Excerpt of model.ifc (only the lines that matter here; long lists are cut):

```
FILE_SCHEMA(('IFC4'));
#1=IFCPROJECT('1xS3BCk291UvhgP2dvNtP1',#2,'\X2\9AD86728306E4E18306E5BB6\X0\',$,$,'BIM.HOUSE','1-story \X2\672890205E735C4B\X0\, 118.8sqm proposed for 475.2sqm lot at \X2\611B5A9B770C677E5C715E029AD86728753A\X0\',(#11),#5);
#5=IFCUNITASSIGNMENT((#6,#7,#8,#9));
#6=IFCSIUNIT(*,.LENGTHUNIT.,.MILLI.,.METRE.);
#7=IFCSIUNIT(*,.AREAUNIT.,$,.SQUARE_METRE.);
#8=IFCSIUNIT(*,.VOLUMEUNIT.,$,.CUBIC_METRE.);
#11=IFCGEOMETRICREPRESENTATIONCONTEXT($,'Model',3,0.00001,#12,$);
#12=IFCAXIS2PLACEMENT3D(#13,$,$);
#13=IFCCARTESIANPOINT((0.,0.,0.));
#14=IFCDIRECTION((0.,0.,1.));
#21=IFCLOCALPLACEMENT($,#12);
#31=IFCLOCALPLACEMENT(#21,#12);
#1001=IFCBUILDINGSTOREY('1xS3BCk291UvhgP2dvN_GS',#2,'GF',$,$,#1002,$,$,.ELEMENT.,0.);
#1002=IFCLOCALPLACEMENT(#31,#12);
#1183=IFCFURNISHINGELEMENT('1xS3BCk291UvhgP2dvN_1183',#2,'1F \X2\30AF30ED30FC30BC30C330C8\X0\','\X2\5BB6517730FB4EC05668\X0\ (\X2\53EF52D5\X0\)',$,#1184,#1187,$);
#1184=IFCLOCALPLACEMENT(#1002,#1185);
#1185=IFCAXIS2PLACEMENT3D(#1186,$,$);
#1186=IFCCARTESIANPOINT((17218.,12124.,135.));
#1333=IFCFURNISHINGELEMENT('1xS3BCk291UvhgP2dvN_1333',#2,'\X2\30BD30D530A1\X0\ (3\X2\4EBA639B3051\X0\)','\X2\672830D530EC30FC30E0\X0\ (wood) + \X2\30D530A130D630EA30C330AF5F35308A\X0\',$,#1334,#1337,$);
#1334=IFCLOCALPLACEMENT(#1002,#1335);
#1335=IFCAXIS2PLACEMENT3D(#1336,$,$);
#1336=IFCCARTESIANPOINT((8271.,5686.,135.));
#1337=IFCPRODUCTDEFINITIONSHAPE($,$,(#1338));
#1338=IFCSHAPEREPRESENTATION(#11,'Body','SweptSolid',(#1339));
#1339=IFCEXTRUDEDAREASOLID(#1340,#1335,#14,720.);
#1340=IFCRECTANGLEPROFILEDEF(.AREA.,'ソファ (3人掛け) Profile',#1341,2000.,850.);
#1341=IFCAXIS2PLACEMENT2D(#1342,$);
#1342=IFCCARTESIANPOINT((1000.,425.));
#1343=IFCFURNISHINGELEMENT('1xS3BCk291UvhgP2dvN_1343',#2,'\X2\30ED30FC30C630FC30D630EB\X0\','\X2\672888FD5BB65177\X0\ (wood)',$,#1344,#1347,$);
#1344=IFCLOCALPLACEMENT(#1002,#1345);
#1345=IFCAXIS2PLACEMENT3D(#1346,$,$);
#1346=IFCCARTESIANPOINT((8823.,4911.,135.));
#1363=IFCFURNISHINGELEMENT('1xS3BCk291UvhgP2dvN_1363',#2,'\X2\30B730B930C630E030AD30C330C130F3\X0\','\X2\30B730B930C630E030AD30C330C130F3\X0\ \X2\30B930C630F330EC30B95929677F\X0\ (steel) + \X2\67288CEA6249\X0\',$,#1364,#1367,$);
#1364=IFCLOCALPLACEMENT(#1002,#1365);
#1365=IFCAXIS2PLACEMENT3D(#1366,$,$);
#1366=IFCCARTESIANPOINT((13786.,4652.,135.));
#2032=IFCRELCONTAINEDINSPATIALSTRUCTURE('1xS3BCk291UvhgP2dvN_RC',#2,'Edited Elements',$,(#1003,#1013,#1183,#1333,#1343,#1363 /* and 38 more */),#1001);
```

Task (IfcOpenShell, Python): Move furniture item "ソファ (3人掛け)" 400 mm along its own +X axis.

```python
import ifcopenshell
import ifcopenshell.api.geometry
import ifcopenshell.util.placement
import ifcopenshell.util.unit

model = ifcopenshell.open("model.ifc")
unit_scale = ifcopenshell.util.unit.calculate_unit_scale(model)

item = model.by_guid("1xS3BCk291UvhgP2dvN_1333")
matrix = ifcopenshell.util.placement.get_local_placement(item.ObjectPlacement)
matrix[:3, 3] += matrix[:3, 0] * 0.4 / unit_scale
ifcopenshell.api.geometry.edit_object_placement(model, product=item, matrix=matrix, is_si=False)

print(ifcopenshell.util.placement.get_local_placement(item.ObjectPlacement).round(3) + 0.0)

model.write("model_v2.ifc")
```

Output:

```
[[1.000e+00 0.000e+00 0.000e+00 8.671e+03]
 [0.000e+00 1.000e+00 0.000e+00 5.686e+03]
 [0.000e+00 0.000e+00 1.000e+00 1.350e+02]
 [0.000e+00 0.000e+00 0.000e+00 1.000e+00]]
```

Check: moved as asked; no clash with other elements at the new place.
